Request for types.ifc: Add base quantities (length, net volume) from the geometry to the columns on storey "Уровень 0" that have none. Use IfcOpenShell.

First a look at what the model holds.

```python
import ifcopenshell
import ifcopenshell.util.element
import ifcopenshell.util.unit

model = ifcopenshell.open("types.ifc")
print(model.schema)
for unit_type in ("LENGTHUNIT", "AREAUNIT", "VOLUMEUNIT"):
    print(unit_type, ifcopenshell.util.unit.calculate_unit_scale(model, unit_type))
storey = next(s for s in model.by_type("IfcBuildingStorey") if s.Name == "Уровень 0")
columns = [e for e in ifcopenshell.util.element.get_decomposition(storey) if e.is_a("IfcColumn")]
for e in sorted(columns, key=lambda e: e.id()):
    print(e.id(), e.is_a(), e.Name, list(ifcopenshell.util.element.get_psets(e, qtos_only=True)), sep=" | ")
```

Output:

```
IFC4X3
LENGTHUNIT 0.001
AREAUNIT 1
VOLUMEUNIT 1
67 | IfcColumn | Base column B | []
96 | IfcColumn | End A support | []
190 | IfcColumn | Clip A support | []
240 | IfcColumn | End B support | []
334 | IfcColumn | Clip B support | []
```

```python
import ifcopenshell
import ifcopenshell.api.pset
import ifcopenshell.geom
import ifcopenshell.util.element
import ifcopenshell.util.shape
import ifcopenshell.util.unit

model = ifcopenshell.open("types.ifc")
unit_scale = ifcopenshell.util.unit.calculate_unit_scale(model)
volume_scale = ifcopenshell.util.unit.calculate_unit_scale(model, "VOLUMEUNIT")
settings = ifcopenshell.geom.settings()

storey = next(s for s in model.by_type("IfcBuildingStorey") if s.Name == "Уровень 0")
columns = [e for e in ifcopenshell.util.element.get_decomposition(storey) if e.is_a("IfcColumn")]

for e in sorted(columns, key=lambda e: e.id()):
    if ifcopenshell.util.element.get_psets(e, qtos_only=True, should_inherit=False):
        continue
    # Geometry comes back in metres, in the element's own axes.
    shape = ifcopenshell.geom.create_shape(settings, e)
    values = {
        "Length": ifcopenshell.util.shape.get_z(shape.geometry) / unit_scale,
        "NetVolume": ifcopenshell.util.shape.get_volume(shape.geometry) / volume_scale,
    }
    qto = ifcopenshell.api.pset.add_qto(model, product=e, name="Qto_ColumnBaseQuantities")
    ifcopenshell.api.pset.edit_qto(model, qto=qto, properties=values)
    print(e.id(), {k: round(v, 3) for k, v in values.items()})

model.write("types-out.ifc")
```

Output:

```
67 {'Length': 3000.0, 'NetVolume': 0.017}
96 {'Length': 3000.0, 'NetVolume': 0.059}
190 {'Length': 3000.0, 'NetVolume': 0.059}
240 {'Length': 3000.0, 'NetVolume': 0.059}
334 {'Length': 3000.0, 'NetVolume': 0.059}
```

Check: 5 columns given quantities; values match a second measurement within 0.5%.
